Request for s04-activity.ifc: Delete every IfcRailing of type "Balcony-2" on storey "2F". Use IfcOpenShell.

First a look at what the model holds.

```python
import ifcopenshell
import ifcopenshell.util.element

model = ifcopenshell.open("s04-activity.ifc")
print(model.schema)
storey = next(s for s in model.by_type("IfcBuildingStorey") if s.Name == "2F")
railings = [e for e in ifcopenshell.util.element.get_decomposition(storey) if e.is_a("IfcRailing")]
seen = {}
for e in railings:
    element_type = ifcopenshell.util.element.get_type(e)
    name = element_type.Name if element_type not in (None, e) else None
    seen[name] = seen.get(name, 0) + 1
for name, count in sorted(seen.items(), key=str):
    print(count, "x", name)
```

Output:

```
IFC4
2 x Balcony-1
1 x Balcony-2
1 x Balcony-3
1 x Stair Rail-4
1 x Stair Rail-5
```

```python
import ifcopenshell
import ifcopenshell.api.root
import ifcopenshell.util.element

model = ifcopenshell.open("s04-activity.ifc")

storey = next(s for s in model.by_type("IfcBuildingStorey") if s.Name == "2F")
railings = [e for e in ifcopenshell.util.element.get_decomposition(storey) if e.is_a("IfcRailing")]
targets = [e for e in railings if (t := ifcopenshell.util.element.get_type(e)) not in (None, e) and t.Name == "Balcony-2"]

for e in targets:
    ifcopenshell.api.root.remove_product(model, product=e)
print(len(targets), "removed")

model.write("s04-activity-out.ifc")
```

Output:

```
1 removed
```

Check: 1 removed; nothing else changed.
